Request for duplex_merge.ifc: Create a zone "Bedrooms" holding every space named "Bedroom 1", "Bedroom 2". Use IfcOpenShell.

First a look at what the model holds.

```python
import ifcopenshell

model = ifcopenshell.open("duplex_merge.ifc")
print(model.schema)
seen = {}
for space in model.by_type("IfcSpace"):
    seen[space.LongName] = seen.get(space.LongName, 0) + 1
for name, count in sorted(seen.items(), key=str):
    print(count, "x", name)
print("zones:", [z.Name for z in model.by_type("IfcZone")][:20])
```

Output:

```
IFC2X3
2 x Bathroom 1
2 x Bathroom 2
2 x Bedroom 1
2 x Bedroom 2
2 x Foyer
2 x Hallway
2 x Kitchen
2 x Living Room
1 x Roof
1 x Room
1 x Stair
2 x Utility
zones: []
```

```python
import ifcopenshell
import ifcopenshell.api.group
import ifcopenshell.api.root

model = ifcopenshell.open("duplex_merge.ifc")

names = {"Bedroom 1", "Bedroom 2"}
spaces = [s for s in model.by_type("IfcSpace") if s.LongName in names]

zone = ifcopenshell.api.root.create_entity(model, ifc_class="IfcZone", name="Bedrooms")
ifcopenshell.api.group.assign_group(model, products=spaces, group=zone)
print(len(spaces), "spaces in", zone.Name)

model.write("duplex_merge_rev.ifc")
```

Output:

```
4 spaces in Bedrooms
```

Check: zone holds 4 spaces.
